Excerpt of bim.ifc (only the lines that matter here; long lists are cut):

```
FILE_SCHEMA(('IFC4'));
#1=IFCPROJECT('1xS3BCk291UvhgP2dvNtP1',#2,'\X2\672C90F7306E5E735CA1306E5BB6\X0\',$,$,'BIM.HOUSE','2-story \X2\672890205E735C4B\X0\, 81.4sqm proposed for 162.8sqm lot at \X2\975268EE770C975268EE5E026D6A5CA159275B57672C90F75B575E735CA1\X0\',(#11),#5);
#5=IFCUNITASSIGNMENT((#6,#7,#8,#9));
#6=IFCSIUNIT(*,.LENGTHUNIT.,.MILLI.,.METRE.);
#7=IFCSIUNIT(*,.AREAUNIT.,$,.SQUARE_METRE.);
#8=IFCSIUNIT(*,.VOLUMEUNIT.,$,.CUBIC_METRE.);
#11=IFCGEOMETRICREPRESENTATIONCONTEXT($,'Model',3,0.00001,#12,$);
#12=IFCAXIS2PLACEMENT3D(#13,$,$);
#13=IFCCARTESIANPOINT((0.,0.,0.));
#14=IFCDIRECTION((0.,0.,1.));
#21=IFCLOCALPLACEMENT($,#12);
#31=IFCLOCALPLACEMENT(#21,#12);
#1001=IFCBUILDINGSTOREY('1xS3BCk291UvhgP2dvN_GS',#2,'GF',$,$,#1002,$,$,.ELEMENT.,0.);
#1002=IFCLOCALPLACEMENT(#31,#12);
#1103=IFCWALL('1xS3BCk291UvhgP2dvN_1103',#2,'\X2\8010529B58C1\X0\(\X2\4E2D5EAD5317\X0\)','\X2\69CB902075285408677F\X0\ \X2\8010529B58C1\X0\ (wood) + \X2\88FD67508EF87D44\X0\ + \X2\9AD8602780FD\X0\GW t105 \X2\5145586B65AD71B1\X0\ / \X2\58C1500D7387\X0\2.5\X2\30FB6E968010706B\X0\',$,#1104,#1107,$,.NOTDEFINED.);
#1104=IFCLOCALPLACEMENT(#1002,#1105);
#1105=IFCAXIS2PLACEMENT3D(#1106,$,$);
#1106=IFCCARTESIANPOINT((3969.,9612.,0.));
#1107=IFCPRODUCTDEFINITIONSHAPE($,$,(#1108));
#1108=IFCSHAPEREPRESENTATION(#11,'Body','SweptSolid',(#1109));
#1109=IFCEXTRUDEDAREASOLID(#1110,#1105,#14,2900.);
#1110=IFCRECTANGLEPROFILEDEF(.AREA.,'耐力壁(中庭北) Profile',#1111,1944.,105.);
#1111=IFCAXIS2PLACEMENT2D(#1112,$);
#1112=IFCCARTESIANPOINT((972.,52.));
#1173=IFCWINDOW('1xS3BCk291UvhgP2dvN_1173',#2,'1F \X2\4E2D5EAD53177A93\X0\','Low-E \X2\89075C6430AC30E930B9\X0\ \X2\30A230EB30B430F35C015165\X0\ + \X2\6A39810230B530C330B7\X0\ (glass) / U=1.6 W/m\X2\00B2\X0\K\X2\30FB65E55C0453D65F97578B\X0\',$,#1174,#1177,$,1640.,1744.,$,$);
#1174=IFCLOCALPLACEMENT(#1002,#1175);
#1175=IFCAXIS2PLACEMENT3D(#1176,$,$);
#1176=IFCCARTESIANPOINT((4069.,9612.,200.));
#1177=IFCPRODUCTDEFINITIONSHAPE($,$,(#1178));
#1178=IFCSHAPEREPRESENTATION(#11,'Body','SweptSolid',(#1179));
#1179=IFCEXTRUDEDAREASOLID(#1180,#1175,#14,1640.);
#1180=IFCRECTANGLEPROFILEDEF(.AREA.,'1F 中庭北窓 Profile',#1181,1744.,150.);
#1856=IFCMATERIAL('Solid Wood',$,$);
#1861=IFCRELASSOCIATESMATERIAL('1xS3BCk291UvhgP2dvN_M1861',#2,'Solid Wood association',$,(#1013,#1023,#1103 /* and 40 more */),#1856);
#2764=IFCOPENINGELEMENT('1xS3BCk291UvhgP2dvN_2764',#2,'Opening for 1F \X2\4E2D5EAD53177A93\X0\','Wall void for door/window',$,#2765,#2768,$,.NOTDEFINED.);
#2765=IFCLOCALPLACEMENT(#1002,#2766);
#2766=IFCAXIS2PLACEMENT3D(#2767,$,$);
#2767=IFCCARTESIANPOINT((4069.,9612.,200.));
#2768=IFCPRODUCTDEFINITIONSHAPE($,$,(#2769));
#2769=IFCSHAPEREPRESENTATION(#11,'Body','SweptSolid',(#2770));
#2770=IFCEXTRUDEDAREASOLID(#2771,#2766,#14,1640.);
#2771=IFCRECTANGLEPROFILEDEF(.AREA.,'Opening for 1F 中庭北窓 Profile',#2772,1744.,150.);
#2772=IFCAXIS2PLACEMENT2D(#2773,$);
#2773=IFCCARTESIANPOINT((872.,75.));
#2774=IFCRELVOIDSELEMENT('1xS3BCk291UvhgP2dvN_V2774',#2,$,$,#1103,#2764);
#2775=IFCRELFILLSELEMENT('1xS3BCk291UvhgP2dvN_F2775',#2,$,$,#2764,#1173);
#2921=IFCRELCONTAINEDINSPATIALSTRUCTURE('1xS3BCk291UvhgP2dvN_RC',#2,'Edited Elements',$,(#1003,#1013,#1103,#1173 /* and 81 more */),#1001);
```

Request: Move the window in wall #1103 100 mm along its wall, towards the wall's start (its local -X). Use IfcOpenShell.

```python
import ifcopenshell
import ifcopenshell.api.geometry
import ifcopenshell.util.placement
import ifcopenshell.util.unit

model = ifcopenshell.open("bim.ifc")
unit_scale = ifcopenshell.util.unit.calculate_unit_scale(model)

window = model.by_id(1173)
opening = window.FillsVoids[0].RelatingOpeningElement
wall = opening.VoidsElements[0].RelatingBuildingElement

wall_matrix = ifcopenshell.util.placement.get_local_placement(wall.ObjectPlacement)
shift = wall_matrix[:3, 0] * -0.1 / unit_scale
before = ifcopenshell.util.placement.get_local_placement(window.ObjectPlacement)[:3, 3].copy()

# The window is not placed relative to its opening, so move both.
for product in (opening, window):
    matrix = ifcopenshell.util.placement.get_local_placement(product.ObjectPlacement)
    matrix[:3, 3] += shift
    ifcopenshell.api.geometry.edit_object_placement(model, product=product, matrix=matrix, is_si=False)

after = ifcopenshell.util.placement.get_local_placement(window.ObjectPlacement)[:3, 3]
print("window moved by", (after - before).round(3) + 0.0)

model.write("bim_edited.ifc")
```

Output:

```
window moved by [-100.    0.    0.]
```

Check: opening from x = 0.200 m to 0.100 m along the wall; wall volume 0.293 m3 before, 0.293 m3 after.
